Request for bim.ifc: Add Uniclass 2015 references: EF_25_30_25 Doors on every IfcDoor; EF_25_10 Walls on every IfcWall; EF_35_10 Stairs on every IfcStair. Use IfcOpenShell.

First a look at what the model holds.

```python
import ifcopenshell

model = ifcopenshell.open("bim.ifc")
print(model.schema)
print("classifications:", [c.Name for c in model.by_type("IfcClassification")])
for ifc_class in ("IfcDoor", "IfcRoof", "IfcStair", "IfcWall", "IfcWindow"):
    print(ifc_class, len(model.by_type(ifc_class)))
```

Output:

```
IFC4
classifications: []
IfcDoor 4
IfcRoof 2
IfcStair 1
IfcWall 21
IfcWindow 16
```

```python
import ifcopenshell
import ifcopenshell.api.classification

model = ifcopenshell.open("bim.ifc")

system = ifcopenshell.api.classification.add_classification(model, classification="Uniclass 2015")

codes = {
    "IfcDoor": ("EF_25_30_25", "Doors"),
    "IfcWall": ("EF_25_10", "Walls"),
    "IfcStair": ("EF_35_10", "Stairs"),
}
for ifc_class, (code, name) in codes.items():
    products = model.by_type(ifc_class)
    ifcopenshell.api.classification.add_reference(
        model, products=products, classification=system, identification=code, name=name
    )
    print(code, len(products))

model.write("bim-out.ifc")
```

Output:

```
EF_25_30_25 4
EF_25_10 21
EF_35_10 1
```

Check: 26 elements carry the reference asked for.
